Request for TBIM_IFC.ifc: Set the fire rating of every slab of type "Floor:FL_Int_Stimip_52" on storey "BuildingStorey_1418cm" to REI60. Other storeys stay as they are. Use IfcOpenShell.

First a look at what the model holds.

```python
import ifcopenshell
import ifcopenshell.util.element

model = ifcopenshell.open("TBIM_IFC.ifc")
print(model.schema)
storey = next(s for s in model.by_type("IfcBuildingStorey") if s.Name == "BuildingStorey_1418cm")
slabs = [e for e in ifcopenshell.util.element.get_decomposition(storey) if e.is_a("IfcSlab")]
seen = {}
for e in slabs:
    element_type = ifcopenshell.util.element.get_type(e)
    key = (element_type.Name if element_type != e and element_type else None, ifcopenshell.util.element.get_pset(e, "Pset_SlabCommon", "FireRating"))
    seen[key] = seen.get(key, 0) + 1
for (name, value), count in sorted(seen.items(), key=str):
    print(count, "x", name, "|", value)
```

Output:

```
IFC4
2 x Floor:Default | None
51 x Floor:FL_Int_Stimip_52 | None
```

```python
import ifcopenshell
import ifcopenshell.api.pset
import ifcopenshell.util.element

model = ifcopenshell.open("TBIM_IFC.ifc")

storey = next(s for s in model.by_type("IfcBuildingStorey") if s.Name == "BuildingStorey_1418cm")
slabs = [e for e in ifcopenshell.util.element.get_decomposition(storey) if e.is_a("IfcSlab")]

count = 0
for e in slabs:
    element_type = ifcopenshell.util.element.get_type(e)
    if element_type in (None, e) or element_type.Name != "Floor:FL_Int_Stimip_52":
        continue
    # add_pset returns the element's existing set when there is one.
    pset = ifcopenshell.api.pset.add_pset(model, product=e, name="Pset_SlabCommon")
    ifcopenshell.api.pset.edit_pset(model, pset=pset, properties={"FireRating": "REI60"})
    count += 1

print(count, "slabs updated")

model.write("TBIM_IFC_rev.ifc")
```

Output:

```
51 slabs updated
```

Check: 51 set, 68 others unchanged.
